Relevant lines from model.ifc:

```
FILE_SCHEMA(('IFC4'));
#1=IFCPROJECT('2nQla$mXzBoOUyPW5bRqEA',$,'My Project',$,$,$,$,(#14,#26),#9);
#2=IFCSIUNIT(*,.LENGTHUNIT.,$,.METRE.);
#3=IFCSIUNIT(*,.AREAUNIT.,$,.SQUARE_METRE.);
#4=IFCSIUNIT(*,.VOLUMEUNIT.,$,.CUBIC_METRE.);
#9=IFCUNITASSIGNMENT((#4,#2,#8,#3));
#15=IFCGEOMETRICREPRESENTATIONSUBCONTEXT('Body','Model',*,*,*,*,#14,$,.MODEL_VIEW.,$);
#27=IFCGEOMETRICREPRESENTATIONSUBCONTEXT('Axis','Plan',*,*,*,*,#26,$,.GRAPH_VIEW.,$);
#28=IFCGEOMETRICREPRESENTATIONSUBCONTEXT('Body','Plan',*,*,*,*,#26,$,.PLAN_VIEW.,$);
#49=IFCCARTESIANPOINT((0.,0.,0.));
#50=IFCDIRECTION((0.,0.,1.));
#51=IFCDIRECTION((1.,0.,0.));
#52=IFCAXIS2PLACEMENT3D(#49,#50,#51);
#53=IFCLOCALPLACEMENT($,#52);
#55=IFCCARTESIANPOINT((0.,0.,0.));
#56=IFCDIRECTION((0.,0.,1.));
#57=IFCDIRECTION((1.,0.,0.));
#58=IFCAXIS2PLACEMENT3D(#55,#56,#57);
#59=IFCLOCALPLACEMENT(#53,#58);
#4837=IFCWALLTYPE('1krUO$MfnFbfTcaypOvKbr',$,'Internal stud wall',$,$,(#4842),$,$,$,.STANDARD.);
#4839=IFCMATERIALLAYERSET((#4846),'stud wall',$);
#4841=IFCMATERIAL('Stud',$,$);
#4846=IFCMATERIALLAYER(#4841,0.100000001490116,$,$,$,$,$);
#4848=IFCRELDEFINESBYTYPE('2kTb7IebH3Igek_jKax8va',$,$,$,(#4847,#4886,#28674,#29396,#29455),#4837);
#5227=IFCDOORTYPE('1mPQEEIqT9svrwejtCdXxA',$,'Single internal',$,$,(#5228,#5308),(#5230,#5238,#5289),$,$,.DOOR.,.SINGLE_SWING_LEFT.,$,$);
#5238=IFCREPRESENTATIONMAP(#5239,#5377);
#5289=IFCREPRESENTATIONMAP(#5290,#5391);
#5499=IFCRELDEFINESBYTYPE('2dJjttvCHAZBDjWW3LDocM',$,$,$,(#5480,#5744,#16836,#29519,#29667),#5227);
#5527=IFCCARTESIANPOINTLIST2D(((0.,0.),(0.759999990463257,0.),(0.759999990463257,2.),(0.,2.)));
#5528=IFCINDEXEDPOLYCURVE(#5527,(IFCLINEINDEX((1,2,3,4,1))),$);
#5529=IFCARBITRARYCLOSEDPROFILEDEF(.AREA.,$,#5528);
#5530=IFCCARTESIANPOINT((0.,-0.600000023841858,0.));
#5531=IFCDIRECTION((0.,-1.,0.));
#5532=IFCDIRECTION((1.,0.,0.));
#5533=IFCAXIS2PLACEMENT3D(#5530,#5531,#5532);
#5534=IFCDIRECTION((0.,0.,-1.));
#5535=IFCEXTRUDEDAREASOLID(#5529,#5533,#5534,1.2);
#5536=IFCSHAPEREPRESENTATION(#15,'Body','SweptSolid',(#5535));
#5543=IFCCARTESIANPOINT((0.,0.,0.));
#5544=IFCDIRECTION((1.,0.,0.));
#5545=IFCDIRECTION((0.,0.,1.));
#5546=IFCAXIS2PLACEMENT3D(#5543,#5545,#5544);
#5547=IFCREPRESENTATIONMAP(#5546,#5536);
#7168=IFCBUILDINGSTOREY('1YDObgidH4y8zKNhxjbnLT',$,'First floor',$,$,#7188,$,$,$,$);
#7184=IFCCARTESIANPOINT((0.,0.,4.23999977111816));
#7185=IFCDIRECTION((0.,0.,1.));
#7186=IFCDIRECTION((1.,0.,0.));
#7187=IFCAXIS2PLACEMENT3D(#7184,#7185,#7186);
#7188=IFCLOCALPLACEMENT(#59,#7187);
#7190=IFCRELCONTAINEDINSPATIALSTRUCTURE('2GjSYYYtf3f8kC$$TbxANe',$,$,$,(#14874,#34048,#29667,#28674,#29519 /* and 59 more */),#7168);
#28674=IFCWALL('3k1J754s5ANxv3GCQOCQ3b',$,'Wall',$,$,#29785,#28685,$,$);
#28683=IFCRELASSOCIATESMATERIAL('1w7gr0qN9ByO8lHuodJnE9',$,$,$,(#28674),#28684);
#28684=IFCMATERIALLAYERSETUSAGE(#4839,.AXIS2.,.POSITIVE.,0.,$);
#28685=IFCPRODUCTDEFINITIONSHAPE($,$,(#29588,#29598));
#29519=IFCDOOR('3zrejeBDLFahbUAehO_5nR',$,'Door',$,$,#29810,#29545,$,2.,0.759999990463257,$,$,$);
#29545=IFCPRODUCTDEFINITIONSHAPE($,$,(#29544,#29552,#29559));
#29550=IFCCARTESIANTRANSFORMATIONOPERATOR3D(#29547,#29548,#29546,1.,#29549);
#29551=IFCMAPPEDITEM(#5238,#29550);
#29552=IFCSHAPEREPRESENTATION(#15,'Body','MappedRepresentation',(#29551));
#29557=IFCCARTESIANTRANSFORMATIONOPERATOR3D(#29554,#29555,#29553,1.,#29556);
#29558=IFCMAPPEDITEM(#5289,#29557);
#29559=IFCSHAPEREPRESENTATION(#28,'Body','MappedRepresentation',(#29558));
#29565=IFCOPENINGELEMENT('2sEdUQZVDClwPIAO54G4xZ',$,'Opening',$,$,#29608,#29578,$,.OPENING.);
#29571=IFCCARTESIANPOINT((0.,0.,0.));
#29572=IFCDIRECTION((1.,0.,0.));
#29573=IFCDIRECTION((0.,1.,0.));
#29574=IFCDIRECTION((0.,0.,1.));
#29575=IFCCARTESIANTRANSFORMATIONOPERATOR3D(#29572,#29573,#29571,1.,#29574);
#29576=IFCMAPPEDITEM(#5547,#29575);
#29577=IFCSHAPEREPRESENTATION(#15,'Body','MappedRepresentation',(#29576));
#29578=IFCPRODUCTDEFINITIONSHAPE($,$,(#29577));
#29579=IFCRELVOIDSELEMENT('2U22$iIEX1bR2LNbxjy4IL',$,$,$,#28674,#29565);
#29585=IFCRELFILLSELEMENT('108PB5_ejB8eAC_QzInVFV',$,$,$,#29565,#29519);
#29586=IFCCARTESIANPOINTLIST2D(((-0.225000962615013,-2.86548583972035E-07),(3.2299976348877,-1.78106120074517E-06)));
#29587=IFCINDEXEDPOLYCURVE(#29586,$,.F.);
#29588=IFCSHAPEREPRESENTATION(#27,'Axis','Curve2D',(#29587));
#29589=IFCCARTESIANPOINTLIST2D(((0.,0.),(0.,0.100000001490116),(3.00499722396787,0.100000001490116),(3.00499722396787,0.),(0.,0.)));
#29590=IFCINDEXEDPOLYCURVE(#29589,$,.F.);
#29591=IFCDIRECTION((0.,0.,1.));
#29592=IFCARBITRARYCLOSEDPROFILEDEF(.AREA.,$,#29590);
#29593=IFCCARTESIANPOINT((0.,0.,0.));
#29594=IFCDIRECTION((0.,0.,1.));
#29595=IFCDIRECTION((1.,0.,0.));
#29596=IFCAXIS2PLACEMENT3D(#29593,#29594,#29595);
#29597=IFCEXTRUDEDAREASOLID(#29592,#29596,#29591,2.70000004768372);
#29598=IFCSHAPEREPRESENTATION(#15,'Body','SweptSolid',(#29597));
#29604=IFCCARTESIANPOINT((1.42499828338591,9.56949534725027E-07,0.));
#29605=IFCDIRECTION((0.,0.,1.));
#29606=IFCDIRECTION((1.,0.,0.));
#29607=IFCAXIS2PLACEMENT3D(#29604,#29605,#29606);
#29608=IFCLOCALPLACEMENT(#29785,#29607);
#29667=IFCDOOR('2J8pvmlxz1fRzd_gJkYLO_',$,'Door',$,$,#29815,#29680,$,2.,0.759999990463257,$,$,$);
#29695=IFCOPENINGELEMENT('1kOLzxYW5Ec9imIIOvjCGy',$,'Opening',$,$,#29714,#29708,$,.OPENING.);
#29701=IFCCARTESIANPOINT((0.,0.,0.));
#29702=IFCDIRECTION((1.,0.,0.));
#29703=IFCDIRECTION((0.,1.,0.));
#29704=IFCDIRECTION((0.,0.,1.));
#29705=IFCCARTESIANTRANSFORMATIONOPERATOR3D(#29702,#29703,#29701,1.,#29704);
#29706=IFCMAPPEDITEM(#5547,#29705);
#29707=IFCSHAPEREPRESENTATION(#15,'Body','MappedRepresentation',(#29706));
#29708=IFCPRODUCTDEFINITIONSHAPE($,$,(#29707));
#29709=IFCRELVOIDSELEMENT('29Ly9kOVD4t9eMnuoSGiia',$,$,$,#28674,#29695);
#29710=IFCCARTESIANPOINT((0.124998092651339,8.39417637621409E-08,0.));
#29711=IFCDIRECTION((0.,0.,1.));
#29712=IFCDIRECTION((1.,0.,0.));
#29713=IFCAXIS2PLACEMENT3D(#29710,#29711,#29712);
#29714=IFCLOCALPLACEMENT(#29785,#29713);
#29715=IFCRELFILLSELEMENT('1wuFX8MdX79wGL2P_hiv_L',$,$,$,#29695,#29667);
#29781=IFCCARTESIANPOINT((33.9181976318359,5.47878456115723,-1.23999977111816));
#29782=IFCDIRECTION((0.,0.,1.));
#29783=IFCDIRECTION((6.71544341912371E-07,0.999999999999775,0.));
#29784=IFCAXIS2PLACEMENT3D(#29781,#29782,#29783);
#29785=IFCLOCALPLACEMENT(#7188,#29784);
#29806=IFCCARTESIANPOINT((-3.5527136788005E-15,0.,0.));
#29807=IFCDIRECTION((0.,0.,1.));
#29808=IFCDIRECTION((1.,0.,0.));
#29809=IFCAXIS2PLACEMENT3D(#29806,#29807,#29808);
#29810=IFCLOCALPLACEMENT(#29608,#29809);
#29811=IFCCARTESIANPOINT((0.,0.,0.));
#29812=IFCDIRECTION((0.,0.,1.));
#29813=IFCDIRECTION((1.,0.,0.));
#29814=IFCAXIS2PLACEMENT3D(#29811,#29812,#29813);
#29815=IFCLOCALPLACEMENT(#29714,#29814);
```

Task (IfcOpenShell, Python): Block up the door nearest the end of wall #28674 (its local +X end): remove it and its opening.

```python
import ifcopenshell
import ifcopenshell.api.feature
import ifcopenshell.api.root
import ifcopenshell.geom
import ifcopenshell.util.shape

model = ifcopenshell.open("model.ifc")
settings = ifcopenshell.geom.settings()


def volume(element):
    """Net volume in cubic metres, openings subtracted."""
    shape = ifcopenshell.geom.create_shape(settings, element)
    return ifcopenshell.util.shape.get_volume(shape.geometry)


door = model.by_guid("3zrejeBDLFahbUAehO_5nR")
opening = door.FillsVoids[0].RelatingOpeningElement
wall = opening.VoidsElements[0].RelatingBuildingElement
before = volume(wall)

ifcopenshell.api.root.remove_product(model, product=door)
ifcopenshell.api.feature.remove_feature(model, feature=opening)

after = volume(wall)

print(f"wall volume {before:.3f} -> {after:.3f} m3")

model.write("model_rev.ifc")
```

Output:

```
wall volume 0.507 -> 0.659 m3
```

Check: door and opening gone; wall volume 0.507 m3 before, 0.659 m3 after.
